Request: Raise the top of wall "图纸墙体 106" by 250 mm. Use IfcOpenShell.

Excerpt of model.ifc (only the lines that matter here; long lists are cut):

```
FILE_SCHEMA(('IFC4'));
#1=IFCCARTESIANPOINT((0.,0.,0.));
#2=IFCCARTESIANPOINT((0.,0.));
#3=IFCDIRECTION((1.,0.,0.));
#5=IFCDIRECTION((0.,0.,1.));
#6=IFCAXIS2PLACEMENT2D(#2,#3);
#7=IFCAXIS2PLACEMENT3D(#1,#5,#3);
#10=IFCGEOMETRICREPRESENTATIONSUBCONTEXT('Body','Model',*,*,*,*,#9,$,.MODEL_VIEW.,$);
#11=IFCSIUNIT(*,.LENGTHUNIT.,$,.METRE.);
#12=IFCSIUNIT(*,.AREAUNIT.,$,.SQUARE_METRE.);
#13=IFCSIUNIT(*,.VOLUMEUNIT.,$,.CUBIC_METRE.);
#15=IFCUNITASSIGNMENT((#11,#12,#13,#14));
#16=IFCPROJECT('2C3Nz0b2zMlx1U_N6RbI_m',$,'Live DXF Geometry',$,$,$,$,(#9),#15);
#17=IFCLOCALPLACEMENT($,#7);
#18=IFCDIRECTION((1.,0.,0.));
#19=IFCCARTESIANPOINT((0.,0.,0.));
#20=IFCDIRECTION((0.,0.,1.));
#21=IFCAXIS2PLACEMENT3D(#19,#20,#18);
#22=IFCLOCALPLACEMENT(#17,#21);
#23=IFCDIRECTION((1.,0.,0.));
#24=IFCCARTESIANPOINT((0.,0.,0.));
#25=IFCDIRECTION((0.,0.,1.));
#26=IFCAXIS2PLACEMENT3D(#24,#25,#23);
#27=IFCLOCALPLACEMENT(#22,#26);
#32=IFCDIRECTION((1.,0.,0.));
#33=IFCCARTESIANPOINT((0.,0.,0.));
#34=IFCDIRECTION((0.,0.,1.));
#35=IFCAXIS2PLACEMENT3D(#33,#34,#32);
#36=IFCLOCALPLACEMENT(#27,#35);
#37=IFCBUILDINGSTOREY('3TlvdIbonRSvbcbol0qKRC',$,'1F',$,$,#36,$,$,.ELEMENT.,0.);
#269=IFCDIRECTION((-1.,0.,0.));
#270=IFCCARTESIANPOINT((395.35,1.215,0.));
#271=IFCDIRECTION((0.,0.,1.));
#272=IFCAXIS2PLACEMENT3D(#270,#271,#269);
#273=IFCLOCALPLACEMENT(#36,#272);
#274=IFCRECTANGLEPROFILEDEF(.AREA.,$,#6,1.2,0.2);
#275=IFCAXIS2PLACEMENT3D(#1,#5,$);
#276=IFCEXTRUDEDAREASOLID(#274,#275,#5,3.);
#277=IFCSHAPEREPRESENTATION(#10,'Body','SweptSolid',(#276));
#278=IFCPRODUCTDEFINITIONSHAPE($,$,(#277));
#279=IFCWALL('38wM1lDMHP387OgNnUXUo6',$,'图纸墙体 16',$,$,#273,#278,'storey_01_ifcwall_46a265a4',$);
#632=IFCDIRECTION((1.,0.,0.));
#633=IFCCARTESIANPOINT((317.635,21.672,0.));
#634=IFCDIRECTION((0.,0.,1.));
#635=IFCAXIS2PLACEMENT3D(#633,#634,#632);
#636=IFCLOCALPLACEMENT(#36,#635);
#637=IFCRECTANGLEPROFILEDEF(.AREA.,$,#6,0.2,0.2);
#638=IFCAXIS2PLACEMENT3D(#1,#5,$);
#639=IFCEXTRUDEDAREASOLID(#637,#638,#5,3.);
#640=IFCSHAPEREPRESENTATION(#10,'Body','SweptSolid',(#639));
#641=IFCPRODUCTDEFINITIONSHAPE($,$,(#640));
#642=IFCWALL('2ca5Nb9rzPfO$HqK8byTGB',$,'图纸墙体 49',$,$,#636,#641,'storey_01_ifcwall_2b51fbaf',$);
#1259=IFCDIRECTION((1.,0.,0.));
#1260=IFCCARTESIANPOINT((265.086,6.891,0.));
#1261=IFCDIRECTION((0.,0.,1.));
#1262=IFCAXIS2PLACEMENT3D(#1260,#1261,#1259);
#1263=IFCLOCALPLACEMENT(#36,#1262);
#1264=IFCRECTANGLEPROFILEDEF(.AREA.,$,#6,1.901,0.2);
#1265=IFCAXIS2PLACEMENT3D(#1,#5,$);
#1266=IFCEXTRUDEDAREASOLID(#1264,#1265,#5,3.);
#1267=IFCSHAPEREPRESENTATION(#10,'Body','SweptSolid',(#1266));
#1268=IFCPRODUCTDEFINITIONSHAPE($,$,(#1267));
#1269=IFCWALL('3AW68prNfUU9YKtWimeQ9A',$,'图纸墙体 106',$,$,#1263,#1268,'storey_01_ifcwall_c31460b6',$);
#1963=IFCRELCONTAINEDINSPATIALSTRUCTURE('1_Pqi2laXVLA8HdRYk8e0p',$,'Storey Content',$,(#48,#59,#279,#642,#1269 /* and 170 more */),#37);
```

```python
import ifcopenshell
import ifcopenshell.geom
import ifcopenshell.util.representation
import ifcopenshell.util.shape
import ifcopenshell.util.unit

model = ifcopenshell.open("model.ifc")
unit_scale = ifcopenshell.util.unit.calculate_unit_scale(model)
settings = ifcopenshell.geom.settings()


def volume(element):
    """Net volume in cubic metres, openings subtracted."""
    shape = ifcopenshell.geom.create_shape(settings, element)
    return ifcopenshell.util.shape.get_volume(shape.geometry)


wall = model.by_guid("3AW68prNfUU9YKtWimeQ9A")
before = volume(wall)

body = ifcopenshell.util.representation.get_representation(wall, "Model", "Body")
solid = body.Items[0]
old_height = solid.Depth
solid.Depth += 0.25 / unit_scale
after = volume(wall)

print(f"height {old_height:g} -> {solid.Depth:g}, volume {before:.3f} -> {after:.3f} m3")

model.write("model_edited.ifc")
```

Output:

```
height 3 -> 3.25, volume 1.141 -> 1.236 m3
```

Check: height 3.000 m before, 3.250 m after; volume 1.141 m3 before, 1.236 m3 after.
